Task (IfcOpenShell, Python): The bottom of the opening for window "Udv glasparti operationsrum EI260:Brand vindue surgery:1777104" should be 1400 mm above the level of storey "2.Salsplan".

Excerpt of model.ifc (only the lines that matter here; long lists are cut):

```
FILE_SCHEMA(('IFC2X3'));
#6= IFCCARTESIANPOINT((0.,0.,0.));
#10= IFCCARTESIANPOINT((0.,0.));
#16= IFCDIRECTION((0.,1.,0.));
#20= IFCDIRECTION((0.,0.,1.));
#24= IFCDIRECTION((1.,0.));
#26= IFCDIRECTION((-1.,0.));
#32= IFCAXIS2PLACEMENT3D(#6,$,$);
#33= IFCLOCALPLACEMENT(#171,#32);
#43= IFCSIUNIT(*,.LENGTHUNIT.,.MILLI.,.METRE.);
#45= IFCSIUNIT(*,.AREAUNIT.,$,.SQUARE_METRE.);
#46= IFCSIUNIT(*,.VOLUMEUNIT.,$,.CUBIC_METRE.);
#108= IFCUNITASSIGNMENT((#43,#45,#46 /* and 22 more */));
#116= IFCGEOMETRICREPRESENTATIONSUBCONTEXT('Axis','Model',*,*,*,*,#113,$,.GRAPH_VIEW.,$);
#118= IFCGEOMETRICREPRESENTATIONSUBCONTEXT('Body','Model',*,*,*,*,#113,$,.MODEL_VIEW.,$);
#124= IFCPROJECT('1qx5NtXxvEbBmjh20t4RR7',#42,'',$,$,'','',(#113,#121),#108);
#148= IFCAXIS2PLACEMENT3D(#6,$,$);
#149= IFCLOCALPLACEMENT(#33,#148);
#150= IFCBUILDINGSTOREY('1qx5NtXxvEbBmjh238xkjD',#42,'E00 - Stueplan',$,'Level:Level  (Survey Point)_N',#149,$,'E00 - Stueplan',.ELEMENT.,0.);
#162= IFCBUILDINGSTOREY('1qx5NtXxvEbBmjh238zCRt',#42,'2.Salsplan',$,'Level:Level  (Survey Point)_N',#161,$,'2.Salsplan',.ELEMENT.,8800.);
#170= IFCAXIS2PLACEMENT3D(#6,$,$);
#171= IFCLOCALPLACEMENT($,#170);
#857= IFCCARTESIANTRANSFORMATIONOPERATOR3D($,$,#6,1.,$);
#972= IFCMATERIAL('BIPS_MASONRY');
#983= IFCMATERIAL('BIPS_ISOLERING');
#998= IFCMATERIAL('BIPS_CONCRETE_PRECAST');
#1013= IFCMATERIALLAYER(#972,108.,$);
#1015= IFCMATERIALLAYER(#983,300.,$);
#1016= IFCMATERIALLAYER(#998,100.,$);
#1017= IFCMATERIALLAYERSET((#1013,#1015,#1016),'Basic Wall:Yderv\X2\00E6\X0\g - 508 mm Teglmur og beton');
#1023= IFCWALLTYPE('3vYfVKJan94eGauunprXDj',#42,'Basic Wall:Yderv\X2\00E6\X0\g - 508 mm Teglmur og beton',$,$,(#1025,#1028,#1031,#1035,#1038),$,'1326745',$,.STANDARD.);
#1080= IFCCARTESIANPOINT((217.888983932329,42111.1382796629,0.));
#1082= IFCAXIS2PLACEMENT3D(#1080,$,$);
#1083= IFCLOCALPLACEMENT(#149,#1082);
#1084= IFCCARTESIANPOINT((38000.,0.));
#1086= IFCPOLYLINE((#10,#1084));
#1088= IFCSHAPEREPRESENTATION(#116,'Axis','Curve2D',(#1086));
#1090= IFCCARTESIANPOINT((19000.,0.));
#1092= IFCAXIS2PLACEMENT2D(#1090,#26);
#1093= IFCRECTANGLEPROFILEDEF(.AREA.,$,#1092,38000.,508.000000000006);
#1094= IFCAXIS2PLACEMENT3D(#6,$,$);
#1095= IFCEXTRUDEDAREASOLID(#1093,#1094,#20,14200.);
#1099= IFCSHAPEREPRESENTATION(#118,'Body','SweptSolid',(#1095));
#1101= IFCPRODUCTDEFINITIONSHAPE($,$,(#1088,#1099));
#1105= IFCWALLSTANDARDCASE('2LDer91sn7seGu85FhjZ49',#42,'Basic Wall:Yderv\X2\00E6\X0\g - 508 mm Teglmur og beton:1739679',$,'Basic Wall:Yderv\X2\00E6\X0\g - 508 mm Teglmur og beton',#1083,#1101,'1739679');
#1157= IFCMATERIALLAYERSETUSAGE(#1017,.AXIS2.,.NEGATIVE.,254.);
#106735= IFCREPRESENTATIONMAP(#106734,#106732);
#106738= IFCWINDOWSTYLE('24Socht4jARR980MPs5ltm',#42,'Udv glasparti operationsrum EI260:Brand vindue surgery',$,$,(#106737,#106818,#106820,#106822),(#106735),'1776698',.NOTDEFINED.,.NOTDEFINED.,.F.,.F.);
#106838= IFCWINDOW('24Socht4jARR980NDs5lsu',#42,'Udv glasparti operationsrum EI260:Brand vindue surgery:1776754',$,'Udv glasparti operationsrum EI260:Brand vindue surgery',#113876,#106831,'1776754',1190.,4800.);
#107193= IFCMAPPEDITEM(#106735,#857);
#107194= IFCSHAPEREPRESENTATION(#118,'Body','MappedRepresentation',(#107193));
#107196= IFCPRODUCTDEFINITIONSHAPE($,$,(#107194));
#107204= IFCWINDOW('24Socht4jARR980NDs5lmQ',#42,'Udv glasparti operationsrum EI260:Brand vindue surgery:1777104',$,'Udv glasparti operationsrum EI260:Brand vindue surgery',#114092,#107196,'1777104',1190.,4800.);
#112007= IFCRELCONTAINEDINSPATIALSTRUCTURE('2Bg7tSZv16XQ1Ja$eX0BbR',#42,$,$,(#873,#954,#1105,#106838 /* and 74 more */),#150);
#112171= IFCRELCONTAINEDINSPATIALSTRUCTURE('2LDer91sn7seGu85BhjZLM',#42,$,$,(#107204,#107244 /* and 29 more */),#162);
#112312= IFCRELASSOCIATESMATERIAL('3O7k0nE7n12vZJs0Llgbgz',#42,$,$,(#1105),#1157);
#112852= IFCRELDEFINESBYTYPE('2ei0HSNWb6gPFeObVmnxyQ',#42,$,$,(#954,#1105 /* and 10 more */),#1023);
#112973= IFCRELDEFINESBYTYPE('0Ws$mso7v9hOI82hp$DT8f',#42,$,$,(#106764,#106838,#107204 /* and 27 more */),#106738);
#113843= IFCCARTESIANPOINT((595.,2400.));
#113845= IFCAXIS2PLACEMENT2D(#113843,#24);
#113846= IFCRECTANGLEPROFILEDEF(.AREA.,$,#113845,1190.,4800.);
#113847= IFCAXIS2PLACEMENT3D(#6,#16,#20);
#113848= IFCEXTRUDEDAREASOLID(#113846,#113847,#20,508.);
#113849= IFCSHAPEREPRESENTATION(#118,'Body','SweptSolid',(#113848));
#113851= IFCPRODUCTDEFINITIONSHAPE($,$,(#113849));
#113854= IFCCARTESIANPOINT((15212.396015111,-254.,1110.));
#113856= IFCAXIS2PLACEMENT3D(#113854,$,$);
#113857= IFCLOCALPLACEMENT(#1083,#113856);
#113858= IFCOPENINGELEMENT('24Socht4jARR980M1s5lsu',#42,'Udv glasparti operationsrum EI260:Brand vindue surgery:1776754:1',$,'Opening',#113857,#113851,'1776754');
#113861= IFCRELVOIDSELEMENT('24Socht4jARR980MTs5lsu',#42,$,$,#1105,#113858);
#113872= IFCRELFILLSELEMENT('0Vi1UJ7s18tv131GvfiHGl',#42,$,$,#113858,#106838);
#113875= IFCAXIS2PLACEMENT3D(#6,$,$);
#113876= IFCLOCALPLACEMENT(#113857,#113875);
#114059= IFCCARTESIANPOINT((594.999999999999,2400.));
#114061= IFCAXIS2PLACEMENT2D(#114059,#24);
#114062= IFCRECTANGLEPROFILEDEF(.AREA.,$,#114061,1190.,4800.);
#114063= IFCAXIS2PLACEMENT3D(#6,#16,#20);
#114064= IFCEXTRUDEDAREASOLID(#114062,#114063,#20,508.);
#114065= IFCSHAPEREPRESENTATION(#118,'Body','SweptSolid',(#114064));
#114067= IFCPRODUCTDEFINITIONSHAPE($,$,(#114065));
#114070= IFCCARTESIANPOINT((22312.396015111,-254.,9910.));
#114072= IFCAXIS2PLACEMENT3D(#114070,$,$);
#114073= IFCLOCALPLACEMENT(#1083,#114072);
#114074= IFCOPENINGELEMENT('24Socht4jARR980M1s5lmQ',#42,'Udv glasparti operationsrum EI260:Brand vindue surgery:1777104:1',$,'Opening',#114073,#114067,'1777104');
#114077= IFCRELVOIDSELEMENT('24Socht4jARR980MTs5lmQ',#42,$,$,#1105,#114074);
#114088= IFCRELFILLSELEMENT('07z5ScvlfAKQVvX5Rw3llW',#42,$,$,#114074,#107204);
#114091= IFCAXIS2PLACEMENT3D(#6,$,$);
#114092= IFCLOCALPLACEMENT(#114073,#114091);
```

```python
import numpy as np
import ifcopenshell
import ifcopenshell.api.geometry
import ifcopenshell.geom
import ifcopenshell.util.element
import ifcopenshell.util.placement
import ifcopenshell.util.shape
import ifcopenshell.util.unit

model = ifcopenshell.open("model.ifc")
unit_scale = ifcopenshell.util.unit.calculate_unit_scale(model)

window = model.by_guid("24Socht4jARR980NDs5lmQ")
opening = window.FillsVoids[0].RelatingOpeningElement
storey = ifcopenshell.util.element.get_container(window, ifc_class="IfcBuildingStorey")
level = ifcopenshell.util.placement.get_local_placement(storey.ObjectPlacement)[2, 3]

# The opening's origin need not be at the sill, so measure its lowest point.
shape = ifcopenshell.geom.create_shape(ifcopenshell.geom.settings(), opening)
bottom = ifcopenshell.util.shape.get_shape_bottom_elevation(shape, shape.geometry) / unit_scale
dz = level + 1.4 / unit_scale - bottom

shift = np.array([0.0, 0.0, dz])
# The window is placed relative to its opening, so it follows when the opening moves.
matrix = ifcopenshell.util.placement.get_local_placement(opening.ObjectPlacement)
matrix[:3, 3] += shift
ifcopenshell.api.geometry.edit_object_placement(
    model, product=opening, matrix=matrix, is_si=False, should_transform_children=True
)

print(f"moved by {dz * unit_scale:+.3f} m")

model.write("model-out.ifc")
```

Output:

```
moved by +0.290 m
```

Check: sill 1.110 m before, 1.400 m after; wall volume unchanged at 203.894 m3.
